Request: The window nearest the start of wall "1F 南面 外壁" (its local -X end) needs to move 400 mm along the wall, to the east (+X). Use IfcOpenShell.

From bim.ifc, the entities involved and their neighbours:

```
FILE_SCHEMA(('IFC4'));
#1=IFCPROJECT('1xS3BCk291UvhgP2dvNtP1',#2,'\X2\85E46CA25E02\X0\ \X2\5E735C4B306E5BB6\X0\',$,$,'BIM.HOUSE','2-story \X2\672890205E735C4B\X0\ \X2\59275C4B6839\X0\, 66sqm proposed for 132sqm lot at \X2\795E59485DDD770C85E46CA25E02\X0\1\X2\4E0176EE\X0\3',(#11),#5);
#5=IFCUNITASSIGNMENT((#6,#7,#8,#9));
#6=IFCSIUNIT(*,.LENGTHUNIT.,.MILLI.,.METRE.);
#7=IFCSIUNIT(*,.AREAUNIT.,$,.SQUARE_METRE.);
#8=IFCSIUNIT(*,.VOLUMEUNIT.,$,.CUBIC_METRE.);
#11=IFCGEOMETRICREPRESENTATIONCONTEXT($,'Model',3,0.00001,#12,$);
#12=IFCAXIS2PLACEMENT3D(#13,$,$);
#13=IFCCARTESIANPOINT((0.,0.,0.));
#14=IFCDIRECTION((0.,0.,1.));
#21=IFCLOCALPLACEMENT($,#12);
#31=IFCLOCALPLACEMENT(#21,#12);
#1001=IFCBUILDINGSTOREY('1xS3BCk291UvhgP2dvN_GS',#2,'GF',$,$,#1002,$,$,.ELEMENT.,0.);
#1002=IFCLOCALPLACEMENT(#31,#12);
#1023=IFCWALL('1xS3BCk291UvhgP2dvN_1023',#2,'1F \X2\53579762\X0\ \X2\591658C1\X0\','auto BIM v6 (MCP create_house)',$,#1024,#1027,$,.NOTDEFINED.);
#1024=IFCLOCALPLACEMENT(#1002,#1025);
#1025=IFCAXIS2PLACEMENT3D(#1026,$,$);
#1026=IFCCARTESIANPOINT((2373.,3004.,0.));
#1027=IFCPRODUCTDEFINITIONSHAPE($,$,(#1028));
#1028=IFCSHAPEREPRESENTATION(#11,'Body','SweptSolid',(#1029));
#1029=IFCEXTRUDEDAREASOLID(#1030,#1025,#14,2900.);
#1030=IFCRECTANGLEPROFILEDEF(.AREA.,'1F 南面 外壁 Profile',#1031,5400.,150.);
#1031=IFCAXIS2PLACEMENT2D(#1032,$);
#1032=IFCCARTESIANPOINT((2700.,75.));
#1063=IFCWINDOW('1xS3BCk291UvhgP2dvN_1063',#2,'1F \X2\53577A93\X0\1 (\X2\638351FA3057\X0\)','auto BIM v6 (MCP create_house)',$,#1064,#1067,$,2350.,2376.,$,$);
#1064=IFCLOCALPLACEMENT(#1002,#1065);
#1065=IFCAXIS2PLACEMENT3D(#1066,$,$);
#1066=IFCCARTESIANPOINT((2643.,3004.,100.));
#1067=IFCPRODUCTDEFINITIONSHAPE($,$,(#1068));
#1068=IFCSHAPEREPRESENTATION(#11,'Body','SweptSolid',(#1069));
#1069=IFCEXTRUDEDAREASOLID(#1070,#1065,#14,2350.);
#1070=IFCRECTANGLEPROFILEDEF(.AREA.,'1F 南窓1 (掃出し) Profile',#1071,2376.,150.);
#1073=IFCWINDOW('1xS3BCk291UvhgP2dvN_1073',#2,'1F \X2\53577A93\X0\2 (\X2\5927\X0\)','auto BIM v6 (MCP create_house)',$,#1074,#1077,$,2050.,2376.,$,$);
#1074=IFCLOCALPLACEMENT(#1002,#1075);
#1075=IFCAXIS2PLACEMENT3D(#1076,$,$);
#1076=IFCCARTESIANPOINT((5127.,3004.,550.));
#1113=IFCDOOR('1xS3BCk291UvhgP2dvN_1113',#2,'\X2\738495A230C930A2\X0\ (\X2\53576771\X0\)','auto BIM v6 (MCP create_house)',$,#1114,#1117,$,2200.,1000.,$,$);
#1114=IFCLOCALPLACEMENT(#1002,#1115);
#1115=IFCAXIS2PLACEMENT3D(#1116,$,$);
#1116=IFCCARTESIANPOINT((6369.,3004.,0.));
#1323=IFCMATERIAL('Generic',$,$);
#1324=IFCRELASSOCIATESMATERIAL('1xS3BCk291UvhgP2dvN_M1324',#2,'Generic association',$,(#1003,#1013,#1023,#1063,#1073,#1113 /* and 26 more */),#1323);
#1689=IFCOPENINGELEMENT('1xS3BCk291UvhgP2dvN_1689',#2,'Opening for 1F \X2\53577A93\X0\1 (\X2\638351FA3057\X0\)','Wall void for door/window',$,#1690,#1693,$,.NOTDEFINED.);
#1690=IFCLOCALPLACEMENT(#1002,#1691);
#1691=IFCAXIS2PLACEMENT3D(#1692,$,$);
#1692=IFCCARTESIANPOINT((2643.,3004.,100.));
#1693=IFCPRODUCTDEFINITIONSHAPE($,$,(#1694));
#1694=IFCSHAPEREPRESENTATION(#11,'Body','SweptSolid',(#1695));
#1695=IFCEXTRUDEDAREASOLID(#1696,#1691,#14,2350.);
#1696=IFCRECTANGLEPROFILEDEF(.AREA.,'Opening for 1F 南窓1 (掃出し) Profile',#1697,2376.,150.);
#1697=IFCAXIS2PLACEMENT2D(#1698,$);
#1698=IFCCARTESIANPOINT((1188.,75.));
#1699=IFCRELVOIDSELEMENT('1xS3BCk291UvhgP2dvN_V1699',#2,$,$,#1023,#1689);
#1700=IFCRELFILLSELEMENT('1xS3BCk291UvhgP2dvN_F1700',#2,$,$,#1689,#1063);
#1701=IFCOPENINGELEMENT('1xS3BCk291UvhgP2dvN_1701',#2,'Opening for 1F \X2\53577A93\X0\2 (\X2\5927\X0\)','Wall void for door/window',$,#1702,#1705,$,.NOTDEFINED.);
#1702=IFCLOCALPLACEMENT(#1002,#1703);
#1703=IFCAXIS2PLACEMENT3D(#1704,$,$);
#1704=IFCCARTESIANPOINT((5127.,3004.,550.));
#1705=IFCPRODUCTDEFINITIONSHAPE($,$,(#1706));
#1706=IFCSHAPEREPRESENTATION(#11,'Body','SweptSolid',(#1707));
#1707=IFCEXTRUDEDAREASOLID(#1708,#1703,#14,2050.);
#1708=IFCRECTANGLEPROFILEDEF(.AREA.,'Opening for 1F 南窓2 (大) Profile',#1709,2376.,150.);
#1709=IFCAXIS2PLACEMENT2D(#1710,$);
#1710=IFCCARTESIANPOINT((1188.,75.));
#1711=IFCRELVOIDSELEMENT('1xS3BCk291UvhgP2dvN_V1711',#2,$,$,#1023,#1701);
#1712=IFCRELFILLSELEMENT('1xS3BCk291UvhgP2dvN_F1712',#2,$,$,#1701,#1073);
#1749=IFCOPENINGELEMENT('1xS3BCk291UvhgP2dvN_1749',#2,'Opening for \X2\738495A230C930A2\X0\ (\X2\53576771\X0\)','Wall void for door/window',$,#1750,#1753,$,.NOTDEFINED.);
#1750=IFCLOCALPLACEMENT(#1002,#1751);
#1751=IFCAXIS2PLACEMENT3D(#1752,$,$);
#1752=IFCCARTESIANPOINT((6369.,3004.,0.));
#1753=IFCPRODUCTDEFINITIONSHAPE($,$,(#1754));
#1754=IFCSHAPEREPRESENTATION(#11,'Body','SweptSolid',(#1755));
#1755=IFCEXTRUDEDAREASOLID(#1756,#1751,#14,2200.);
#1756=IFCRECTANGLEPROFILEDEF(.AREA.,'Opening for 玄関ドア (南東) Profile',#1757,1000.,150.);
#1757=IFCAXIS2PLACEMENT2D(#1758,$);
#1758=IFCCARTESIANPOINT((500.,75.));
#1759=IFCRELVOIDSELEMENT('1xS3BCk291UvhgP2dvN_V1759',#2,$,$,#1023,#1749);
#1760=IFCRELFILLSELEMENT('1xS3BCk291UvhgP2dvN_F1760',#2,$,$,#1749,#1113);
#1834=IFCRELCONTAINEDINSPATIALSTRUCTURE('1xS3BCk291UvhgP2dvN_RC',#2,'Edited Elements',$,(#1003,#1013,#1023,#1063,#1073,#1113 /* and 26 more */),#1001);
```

```python
import ifcopenshell
import ifcopenshell.api.geometry
import ifcopenshell.util.placement
import ifcopenshell.util.unit

model = ifcopenshell.open("bim.ifc")
unit_scale = ifcopenshell.util.unit.calculate_unit_scale(model)

window = model.by_id(1063)
opening = window.FillsVoids[0].RelatingOpeningElement
wall = opening.VoidsElements[0].RelatingBuildingElement

wall_matrix = ifcopenshell.util.placement.get_local_placement(wall.ObjectPlacement)
shift = wall_matrix[:3, 0] * 0.4 / unit_scale
before = ifcopenshell.util.placement.get_local_placement(window.ObjectPlacement)[:3, 3].copy()

# The window is not placed relative to its opening, so move both.
for product in (opening, window):
    matrix = ifcopenshell.util.placement.get_local_placement(product.ObjectPlacement)
    matrix[:3, 3] += shift
    ifcopenshell.api.geometry.edit_object_placement(model, product=product, matrix=matrix, is_si=False)

after = ifcopenshell.util.placement.get_local_placement(window.ObjectPlacement)[:3, 3]
print("window moved by", (after - before).round(3) + 0.0)

model.write("bim_rev.ifc")
```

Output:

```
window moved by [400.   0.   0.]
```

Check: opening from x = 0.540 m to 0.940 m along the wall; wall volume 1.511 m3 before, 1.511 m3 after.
